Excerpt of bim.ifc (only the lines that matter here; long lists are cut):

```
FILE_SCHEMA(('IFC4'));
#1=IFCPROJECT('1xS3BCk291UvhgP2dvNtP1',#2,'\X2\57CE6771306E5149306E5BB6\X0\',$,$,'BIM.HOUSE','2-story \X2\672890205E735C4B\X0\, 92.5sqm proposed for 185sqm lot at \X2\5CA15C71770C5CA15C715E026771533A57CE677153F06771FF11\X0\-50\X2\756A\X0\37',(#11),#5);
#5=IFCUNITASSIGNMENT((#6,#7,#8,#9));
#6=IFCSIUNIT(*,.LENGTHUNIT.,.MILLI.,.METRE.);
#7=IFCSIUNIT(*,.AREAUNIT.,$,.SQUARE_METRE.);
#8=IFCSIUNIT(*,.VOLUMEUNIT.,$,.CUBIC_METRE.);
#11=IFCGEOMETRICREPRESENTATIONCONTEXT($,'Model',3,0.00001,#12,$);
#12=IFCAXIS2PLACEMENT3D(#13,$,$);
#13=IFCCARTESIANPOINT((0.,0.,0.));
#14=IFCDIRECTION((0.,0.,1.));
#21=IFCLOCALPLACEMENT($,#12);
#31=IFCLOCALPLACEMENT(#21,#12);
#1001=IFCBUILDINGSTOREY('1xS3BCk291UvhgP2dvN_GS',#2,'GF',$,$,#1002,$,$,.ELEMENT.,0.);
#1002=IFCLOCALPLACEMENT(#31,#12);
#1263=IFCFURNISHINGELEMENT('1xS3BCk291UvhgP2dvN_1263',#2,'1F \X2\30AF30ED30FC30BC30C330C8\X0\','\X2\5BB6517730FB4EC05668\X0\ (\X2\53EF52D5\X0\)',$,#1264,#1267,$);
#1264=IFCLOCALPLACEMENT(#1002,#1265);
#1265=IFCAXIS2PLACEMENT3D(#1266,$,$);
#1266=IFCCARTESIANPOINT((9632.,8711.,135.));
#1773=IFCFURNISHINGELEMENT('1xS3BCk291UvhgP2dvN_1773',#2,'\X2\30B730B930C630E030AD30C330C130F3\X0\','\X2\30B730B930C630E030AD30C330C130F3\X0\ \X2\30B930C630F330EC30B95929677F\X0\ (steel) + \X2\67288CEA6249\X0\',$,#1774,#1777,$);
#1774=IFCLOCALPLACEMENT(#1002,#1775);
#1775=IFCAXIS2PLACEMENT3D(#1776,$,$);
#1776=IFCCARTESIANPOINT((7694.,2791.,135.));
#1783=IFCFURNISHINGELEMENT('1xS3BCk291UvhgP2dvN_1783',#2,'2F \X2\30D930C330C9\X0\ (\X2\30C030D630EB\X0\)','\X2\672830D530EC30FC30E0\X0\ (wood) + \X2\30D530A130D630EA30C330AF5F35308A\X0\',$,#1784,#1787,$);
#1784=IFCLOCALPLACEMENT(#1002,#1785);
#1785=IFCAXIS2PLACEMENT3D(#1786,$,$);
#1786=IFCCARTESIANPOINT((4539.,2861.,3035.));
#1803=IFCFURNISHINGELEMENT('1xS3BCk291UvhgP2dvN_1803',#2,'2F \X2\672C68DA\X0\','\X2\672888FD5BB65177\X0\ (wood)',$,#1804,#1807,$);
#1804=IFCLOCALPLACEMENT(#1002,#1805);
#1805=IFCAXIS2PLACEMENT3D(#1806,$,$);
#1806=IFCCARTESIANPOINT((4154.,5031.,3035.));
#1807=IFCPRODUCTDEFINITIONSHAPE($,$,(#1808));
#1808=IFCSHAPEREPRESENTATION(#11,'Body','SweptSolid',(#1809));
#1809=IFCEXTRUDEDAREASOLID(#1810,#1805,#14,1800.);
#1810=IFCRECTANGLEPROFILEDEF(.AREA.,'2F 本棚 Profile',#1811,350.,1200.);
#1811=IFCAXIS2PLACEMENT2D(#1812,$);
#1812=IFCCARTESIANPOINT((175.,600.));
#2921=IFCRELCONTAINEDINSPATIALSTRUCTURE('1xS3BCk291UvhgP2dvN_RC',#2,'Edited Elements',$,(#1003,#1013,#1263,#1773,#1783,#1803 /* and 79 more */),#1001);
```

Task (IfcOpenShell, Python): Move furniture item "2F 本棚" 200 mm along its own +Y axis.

```python
import ifcopenshell
import ifcopenshell.api.geometry
import ifcopenshell.util.placement
import ifcopenshell.util.unit

model = ifcopenshell.open("bim.ifc")
unit_scale = ifcopenshell.util.unit.calculate_unit_scale(model)

item = model.by_guid("1xS3BCk291UvhgP2dvN_1803")
matrix = ifcopenshell.util.placement.get_local_placement(item.ObjectPlacement)
matrix[:3, 3] += matrix[:3, 1] * 0.2 / unit_scale
ifcopenshell.api.geometry.edit_object_placement(model, product=item, matrix=matrix, is_si=False)

print(ifcopenshell.util.placement.get_local_placement(item.ObjectPlacement).round(3) + 0.0)

model.write("bim_updated.ifc")
```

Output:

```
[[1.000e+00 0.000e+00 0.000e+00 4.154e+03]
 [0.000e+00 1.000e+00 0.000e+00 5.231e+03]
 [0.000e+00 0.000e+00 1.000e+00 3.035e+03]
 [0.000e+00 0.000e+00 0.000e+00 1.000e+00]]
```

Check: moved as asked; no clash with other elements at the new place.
